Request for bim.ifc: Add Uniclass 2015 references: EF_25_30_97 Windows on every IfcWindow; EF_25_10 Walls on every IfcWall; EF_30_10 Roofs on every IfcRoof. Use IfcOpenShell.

First a look at what the model holds.

```python
import ifcopenshell

model = ifcopenshell.open("bim.ifc")
print(model.schema)
print("classifications:", [c.Name for c in model.by_type("IfcClassification")])
for ifc_class in ("IfcDoor", "IfcRoof", "IfcStair", "IfcWall", "IfcWindow"):
    print(ifc_class, len(model.by_type(ifc_class)))
```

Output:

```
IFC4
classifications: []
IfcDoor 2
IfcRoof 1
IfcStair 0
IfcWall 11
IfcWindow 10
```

```python
import ifcopenshell
import ifcopenshell.api.classification

model = ifcopenshell.open("bim.ifc")

system = ifcopenshell.api.classification.add_classification(model, classification="Uniclass 2015")

codes = {
    "IfcWindow": ("EF_25_30_97", "Windows"),
    "IfcWall": ("EF_25_10", "Walls"),
    "IfcRoof": ("EF_30_10", "Roofs"),
}
for ifc_class, (code, name) in codes.items():
    products = model.by_type(ifc_class)
    ifcopenshell.api.classification.add_reference(
        model, products=products, classification=system, identification=code, name=name
    )
    print(code, len(products))

model.write("bim_updated.ifc")
```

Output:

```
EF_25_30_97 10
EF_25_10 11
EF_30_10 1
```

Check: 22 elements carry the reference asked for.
